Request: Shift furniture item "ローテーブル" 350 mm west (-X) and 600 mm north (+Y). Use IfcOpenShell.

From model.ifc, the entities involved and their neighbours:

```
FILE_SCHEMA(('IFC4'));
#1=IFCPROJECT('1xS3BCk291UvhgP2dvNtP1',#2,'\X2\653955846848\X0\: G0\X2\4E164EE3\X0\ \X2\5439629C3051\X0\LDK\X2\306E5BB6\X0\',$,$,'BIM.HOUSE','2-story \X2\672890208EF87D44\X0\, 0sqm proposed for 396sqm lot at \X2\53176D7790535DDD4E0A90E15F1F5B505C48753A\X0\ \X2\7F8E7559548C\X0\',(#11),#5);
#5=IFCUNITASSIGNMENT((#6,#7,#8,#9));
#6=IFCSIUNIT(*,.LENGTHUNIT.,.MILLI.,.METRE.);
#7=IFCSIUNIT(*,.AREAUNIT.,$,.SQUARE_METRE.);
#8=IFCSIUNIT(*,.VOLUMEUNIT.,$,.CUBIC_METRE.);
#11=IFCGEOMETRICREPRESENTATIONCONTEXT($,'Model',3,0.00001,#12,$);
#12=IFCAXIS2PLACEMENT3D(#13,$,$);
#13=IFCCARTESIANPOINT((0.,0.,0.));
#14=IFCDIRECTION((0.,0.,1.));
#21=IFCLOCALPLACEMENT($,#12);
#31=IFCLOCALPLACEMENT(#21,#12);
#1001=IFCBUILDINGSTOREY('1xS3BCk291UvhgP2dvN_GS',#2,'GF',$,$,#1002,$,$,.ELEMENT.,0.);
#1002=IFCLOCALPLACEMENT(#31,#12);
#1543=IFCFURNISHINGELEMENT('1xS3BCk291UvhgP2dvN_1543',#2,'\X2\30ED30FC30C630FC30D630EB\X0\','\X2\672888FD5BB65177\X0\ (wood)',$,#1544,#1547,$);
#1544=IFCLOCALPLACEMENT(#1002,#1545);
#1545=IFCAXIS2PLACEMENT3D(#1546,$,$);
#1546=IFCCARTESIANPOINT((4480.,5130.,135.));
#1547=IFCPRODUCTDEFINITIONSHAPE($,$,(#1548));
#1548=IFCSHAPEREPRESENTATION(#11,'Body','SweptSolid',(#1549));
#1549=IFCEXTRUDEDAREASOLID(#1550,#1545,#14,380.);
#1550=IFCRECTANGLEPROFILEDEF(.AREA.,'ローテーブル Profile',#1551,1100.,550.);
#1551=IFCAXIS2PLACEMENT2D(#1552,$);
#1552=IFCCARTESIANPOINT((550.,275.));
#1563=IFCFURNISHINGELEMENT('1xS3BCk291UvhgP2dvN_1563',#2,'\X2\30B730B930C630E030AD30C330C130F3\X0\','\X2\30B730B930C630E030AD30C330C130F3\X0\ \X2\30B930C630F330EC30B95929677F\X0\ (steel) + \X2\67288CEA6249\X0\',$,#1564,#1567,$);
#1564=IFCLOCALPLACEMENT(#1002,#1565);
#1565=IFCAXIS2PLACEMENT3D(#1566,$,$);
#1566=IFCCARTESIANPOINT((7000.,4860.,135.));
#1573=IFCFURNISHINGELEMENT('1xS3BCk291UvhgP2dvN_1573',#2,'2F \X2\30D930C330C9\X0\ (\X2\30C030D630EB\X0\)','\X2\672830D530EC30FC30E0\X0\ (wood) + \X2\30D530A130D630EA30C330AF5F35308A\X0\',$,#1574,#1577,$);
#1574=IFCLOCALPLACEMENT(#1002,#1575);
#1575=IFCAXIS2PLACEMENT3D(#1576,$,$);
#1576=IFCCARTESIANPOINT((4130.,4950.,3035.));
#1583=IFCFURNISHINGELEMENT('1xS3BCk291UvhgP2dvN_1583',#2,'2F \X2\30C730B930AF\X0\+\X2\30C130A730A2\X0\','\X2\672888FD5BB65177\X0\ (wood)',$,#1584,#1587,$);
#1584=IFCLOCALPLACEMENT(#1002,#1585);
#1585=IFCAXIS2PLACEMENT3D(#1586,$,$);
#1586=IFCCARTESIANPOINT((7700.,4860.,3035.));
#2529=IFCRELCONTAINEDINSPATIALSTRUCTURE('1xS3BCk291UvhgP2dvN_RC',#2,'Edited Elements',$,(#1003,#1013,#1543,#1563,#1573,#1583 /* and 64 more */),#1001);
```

```python
import ifcopenshell
import ifcopenshell.api.geometry
import ifcopenshell.util.placement
import ifcopenshell.util.unit

model = ifcopenshell.open("model.ifc")
unit_scale = ifcopenshell.util.unit.calculate_unit_scale(model)

item = model.by_guid("1xS3BCk291UvhgP2dvN_1543")
matrix = ifcopenshell.util.placement.get_local_placement(item.ObjectPlacement)
matrix[0, 3] -= 0.35 / unit_scale
matrix[1, 3] += 0.6 / unit_scale
ifcopenshell.api.geometry.edit_object_placement(model, product=item, matrix=matrix, is_si=False)

print(ifcopenshell.util.placement.get_local_placement(item.ObjectPlacement).round(3) + 0.0)

model.write("model_updated.ifc")
```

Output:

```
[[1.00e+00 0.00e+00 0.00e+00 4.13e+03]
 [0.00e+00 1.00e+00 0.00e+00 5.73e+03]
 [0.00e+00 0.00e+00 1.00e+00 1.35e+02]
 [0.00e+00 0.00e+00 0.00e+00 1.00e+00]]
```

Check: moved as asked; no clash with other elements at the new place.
